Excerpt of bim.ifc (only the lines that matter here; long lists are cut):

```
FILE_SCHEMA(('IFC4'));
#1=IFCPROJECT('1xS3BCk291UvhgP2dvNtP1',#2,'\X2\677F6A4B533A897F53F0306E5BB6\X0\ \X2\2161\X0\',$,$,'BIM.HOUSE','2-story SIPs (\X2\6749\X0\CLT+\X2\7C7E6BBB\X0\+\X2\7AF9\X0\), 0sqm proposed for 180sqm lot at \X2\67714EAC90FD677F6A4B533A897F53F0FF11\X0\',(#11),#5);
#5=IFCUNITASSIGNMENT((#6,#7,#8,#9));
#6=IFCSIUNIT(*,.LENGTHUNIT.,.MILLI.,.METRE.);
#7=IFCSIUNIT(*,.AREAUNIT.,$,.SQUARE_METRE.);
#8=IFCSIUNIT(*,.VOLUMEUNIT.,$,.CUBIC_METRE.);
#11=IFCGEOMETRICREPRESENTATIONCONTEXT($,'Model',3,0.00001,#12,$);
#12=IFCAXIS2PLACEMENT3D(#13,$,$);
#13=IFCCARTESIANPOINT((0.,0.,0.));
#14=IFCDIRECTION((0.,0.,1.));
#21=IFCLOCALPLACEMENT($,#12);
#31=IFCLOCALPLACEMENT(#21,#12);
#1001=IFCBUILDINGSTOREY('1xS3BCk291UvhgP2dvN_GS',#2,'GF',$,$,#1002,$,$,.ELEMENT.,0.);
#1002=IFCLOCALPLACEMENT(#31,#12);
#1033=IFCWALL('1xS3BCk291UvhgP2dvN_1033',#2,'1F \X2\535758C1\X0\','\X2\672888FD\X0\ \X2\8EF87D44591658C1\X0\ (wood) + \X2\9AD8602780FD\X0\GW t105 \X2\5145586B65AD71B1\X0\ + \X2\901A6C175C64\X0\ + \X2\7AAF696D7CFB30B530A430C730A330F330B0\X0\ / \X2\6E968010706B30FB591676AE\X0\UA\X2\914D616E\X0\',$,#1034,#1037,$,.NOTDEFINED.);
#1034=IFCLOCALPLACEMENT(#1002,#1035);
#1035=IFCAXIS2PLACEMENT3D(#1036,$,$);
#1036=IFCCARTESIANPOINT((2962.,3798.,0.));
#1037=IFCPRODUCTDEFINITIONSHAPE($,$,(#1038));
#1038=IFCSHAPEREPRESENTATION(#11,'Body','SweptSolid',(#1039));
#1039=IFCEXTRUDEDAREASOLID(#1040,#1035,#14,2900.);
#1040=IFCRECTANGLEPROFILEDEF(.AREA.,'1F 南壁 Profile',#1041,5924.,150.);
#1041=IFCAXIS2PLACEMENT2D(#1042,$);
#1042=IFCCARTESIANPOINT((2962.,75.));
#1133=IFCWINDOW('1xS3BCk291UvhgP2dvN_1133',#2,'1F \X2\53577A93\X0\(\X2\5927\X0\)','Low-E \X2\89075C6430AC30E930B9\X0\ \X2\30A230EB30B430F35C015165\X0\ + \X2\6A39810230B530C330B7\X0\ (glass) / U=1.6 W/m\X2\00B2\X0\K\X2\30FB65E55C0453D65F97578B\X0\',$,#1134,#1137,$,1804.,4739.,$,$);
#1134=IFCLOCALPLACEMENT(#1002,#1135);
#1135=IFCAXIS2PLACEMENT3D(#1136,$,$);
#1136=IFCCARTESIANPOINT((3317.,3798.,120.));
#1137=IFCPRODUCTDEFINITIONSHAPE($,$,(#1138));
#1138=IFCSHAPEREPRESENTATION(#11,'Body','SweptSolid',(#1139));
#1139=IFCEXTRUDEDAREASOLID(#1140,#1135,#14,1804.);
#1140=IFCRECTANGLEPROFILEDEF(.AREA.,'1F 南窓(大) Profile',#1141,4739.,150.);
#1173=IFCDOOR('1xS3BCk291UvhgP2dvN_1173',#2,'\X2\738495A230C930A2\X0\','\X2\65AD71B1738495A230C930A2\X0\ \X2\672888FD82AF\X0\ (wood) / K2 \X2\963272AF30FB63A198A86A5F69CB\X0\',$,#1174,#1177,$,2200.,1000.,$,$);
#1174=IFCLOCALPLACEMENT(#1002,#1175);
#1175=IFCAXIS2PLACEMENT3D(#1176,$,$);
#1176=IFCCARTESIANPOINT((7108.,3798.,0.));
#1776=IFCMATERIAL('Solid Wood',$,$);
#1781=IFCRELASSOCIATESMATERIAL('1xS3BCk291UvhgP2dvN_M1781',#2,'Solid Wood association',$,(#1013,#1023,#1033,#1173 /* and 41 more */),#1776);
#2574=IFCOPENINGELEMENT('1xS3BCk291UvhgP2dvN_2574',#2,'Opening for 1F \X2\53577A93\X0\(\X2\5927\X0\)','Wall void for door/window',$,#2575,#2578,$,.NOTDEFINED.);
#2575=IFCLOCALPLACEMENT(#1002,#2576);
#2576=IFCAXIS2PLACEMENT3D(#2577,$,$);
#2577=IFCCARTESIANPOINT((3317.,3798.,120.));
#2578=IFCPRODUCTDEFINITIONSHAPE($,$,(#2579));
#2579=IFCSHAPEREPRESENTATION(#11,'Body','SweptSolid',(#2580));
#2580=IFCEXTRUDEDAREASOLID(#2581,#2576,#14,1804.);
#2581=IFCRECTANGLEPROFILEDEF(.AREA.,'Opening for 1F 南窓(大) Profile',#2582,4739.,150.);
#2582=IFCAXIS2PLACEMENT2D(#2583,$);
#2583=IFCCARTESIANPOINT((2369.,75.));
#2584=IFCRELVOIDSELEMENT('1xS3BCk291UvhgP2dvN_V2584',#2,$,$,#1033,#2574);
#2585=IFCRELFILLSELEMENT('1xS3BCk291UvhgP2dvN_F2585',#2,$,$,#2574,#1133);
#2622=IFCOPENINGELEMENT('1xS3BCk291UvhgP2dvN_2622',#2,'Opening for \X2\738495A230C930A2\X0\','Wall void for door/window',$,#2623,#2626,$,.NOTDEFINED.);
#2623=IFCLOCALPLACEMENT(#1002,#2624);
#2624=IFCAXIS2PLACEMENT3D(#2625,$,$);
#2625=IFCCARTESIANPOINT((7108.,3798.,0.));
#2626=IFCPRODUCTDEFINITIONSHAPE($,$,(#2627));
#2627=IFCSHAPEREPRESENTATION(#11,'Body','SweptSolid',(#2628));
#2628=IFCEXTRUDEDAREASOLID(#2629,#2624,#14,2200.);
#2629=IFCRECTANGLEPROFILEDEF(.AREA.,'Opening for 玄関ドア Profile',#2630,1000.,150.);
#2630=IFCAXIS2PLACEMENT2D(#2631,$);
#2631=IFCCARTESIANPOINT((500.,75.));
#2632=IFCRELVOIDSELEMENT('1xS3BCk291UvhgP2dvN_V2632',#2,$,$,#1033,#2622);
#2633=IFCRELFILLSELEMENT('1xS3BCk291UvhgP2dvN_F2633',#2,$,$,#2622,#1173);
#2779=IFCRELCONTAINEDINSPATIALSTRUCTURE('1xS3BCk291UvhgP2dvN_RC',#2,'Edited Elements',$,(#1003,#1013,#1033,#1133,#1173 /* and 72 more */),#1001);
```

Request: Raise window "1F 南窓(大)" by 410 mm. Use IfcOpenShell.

```python
import numpy as np
import ifcopenshell
import ifcopenshell.api.geometry
import ifcopenshell.util.placement
import ifcopenshell.util.unit

model = ifcopenshell.open("bim.ifc")
unit_scale = ifcopenshell.util.unit.calculate_unit_scale(model)

window = model.by_guid("1xS3BCk291UvhgP2dvN_1133")
opening = window.FillsVoids[0].RelatingOpeningElement
dz = 410.0

shift = np.array([0.0, 0.0, dz])
# The window is not placed relative to its opening, so move both.
for product in (opening, window):
    matrix = ifcopenshell.util.placement.get_local_placement(product.ObjectPlacement)
    matrix[:3, 3] += shift
    ifcopenshell.api.geometry.edit_object_placement(model, product=product, matrix=matrix, is_si=False)

print(f"moved by {dz * unit_scale:+.3f} m")

model.write("bim-out.ifc")
```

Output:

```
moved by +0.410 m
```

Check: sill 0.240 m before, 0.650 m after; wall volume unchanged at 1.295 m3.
